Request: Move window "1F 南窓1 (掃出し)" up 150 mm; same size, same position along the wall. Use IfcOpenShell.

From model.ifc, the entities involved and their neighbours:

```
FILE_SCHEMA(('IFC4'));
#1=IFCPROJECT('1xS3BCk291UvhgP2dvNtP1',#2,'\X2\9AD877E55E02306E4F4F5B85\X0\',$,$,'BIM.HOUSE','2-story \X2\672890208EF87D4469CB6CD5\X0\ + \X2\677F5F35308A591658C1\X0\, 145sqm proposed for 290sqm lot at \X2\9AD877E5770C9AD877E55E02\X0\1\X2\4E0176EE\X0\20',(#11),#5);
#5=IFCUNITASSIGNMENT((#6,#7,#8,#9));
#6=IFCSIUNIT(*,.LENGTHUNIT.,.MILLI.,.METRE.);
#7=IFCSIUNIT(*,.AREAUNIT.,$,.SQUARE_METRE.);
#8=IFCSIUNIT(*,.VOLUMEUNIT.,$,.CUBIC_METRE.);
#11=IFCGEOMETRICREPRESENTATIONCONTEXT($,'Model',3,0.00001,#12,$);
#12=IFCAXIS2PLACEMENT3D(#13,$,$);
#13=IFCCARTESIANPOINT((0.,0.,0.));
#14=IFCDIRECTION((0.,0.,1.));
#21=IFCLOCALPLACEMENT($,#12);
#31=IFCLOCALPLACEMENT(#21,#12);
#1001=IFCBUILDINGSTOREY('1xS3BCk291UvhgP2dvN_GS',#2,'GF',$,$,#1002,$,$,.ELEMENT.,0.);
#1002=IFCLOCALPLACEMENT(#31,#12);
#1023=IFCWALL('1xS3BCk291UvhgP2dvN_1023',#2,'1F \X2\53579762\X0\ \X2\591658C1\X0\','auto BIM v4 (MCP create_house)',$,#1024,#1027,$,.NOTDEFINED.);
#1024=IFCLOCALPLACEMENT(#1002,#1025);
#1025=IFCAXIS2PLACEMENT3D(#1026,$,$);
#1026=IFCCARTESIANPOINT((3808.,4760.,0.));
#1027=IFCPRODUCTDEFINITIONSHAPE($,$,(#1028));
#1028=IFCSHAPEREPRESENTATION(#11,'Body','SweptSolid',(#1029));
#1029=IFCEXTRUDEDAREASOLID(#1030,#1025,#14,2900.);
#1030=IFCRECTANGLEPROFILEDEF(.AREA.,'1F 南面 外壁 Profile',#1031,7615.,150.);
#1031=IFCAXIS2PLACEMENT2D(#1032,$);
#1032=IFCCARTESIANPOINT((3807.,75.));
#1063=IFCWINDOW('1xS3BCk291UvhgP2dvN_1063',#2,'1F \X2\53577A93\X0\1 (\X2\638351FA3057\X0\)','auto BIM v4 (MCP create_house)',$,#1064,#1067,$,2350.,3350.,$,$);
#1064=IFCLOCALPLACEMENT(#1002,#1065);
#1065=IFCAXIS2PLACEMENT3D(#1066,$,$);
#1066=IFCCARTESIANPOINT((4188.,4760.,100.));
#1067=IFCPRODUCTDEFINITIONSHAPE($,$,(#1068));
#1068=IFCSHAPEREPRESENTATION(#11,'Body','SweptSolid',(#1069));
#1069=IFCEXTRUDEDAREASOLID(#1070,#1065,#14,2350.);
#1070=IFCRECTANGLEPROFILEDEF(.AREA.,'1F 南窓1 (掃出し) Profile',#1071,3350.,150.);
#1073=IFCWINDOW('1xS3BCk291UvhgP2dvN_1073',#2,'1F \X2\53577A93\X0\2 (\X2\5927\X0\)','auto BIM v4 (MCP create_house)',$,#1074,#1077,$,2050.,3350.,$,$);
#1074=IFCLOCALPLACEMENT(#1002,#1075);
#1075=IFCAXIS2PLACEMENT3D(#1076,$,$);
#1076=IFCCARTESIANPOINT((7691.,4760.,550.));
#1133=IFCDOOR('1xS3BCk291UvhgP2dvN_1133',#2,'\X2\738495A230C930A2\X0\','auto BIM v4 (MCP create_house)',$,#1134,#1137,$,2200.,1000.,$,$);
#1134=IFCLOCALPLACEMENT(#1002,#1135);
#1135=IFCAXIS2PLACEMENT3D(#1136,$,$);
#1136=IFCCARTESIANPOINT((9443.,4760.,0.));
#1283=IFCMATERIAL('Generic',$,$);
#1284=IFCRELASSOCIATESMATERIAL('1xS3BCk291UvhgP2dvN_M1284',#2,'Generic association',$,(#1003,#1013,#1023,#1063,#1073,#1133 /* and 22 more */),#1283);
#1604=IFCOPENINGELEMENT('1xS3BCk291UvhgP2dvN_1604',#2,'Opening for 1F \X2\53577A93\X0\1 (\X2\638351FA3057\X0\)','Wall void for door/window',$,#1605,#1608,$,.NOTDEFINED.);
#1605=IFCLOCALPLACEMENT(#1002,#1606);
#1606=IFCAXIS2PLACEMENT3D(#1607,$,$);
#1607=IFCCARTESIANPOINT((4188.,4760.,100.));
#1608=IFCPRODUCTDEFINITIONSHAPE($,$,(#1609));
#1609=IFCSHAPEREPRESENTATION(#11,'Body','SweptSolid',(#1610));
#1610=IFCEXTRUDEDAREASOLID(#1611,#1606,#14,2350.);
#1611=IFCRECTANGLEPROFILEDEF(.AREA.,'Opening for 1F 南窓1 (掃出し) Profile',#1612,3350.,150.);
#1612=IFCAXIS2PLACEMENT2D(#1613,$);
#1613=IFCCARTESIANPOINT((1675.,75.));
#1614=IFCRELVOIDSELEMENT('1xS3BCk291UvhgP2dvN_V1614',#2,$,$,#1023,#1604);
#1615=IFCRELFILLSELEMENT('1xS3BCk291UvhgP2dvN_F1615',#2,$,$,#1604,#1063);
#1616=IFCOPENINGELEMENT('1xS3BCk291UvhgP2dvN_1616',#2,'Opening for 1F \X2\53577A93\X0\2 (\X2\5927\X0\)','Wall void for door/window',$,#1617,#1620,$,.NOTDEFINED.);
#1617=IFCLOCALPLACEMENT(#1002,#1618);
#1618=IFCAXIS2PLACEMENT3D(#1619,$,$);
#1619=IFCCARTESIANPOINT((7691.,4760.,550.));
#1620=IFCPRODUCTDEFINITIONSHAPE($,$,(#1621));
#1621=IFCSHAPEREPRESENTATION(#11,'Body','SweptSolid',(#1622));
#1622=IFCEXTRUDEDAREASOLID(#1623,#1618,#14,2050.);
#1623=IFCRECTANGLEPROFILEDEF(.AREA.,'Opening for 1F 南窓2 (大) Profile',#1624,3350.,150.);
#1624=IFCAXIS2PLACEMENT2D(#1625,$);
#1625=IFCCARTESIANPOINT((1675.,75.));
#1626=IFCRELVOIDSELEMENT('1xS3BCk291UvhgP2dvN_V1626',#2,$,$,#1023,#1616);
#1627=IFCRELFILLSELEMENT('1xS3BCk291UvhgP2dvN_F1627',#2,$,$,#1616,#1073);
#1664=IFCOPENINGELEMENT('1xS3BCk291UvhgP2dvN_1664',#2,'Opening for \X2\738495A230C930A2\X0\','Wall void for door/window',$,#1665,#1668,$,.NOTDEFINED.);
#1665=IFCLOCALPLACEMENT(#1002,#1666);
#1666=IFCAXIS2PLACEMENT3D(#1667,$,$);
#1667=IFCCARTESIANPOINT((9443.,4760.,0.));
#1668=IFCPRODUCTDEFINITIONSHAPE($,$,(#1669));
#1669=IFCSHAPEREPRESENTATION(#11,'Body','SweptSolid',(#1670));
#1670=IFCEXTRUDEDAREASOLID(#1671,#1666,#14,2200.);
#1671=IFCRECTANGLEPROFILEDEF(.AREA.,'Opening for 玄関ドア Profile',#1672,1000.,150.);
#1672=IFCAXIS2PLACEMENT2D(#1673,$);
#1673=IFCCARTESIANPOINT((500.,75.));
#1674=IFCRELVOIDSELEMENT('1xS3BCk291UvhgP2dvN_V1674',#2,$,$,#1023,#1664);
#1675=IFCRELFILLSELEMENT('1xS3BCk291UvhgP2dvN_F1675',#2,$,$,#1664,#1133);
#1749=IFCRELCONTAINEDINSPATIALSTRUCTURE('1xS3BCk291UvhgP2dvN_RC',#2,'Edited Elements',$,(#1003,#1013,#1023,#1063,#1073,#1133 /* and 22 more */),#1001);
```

```python
import numpy as np
import ifcopenshell
import ifcopenshell.api.geometry
import ifcopenshell.util.placement
import ifcopenshell.util.unit

model = ifcopenshell.open("model.ifc")
unit_scale = ifcopenshell.util.unit.calculate_unit_scale(model)

window = model.by_id(1063)
opening = window.FillsVoids[0].RelatingOpeningElement
dz = 0.15 / unit_scale

shift = np.array([0.0, 0.0, dz])
# The window is not placed relative to its opening, so move both.
for product in (opening, window):
    matrix = ifcopenshell.util.placement.get_local_placement(product.ObjectPlacement)
    matrix[:3, 3] += shift
    ifcopenshell.api.geometry.edit_object_placement(model, product=product, matrix=matrix, is_si=False)

print(f"moved by {dz * unit_scale:+.3f} m")

model.write("model_rev.ifc")
```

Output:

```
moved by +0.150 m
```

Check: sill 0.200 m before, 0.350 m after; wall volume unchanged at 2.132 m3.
